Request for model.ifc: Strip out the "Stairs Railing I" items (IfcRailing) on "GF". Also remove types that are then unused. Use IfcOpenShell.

First a look at what the model holds.

```python
import ifcopenshell
import ifcopenshell.util.element

model = ifcopenshell.open("model.ifc")
print(model.schema)
storey = next(s for s in model.by_type("IfcBuildingStorey") if s.Name == "GF")
railings = [e for e in ifcopenshell.util.element.get_decomposition(storey) if e.is_a("IfcRailing")]
seen = {}
for e in railings:
    element_type = ifcopenshell.util.element.get_type(e)
    name = element_type.Name if element_type not in (None, e) else None
    seen[name] = seen.get(name, 0) + 1
for name, count in sorted(seen.items(), key=str):
    print(count, "x", name)
```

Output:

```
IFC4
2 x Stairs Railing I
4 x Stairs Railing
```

```python
import ifcopenshell
import ifcopenshell.api.root
import ifcopenshell.util.element

model = ifcopenshell.open("model.ifc")

storey = next(s for s in model.by_type("IfcBuildingStorey") if s.Name == "GF")
railings = [e for e in ifcopenshell.util.element.get_decomposition(storey) if e.is_a("IfcRailing")]
targets = [e for e in railings if (t := ifcopenshell.util.element.get_type(e)) not in (None, e) and t.Name == "Stairs Railing I"]
types = {ifcopenshell.util.element.get_type(e) for e in targets} - {None, *targets}

for e in targets:
    ifcopenshell.api.root.remove_product(model, product=e)
print(len(targets), "removed")

unused = [t for t in types if not ifcopenshell.util.element.get_types(t)]
for t in unused:
    ifcopenshell.api.root.remove_product(model, product=t)
print(len(unused), "unused types removed")

model.write("model_rev.ifc")
```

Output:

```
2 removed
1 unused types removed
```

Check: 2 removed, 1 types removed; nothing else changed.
